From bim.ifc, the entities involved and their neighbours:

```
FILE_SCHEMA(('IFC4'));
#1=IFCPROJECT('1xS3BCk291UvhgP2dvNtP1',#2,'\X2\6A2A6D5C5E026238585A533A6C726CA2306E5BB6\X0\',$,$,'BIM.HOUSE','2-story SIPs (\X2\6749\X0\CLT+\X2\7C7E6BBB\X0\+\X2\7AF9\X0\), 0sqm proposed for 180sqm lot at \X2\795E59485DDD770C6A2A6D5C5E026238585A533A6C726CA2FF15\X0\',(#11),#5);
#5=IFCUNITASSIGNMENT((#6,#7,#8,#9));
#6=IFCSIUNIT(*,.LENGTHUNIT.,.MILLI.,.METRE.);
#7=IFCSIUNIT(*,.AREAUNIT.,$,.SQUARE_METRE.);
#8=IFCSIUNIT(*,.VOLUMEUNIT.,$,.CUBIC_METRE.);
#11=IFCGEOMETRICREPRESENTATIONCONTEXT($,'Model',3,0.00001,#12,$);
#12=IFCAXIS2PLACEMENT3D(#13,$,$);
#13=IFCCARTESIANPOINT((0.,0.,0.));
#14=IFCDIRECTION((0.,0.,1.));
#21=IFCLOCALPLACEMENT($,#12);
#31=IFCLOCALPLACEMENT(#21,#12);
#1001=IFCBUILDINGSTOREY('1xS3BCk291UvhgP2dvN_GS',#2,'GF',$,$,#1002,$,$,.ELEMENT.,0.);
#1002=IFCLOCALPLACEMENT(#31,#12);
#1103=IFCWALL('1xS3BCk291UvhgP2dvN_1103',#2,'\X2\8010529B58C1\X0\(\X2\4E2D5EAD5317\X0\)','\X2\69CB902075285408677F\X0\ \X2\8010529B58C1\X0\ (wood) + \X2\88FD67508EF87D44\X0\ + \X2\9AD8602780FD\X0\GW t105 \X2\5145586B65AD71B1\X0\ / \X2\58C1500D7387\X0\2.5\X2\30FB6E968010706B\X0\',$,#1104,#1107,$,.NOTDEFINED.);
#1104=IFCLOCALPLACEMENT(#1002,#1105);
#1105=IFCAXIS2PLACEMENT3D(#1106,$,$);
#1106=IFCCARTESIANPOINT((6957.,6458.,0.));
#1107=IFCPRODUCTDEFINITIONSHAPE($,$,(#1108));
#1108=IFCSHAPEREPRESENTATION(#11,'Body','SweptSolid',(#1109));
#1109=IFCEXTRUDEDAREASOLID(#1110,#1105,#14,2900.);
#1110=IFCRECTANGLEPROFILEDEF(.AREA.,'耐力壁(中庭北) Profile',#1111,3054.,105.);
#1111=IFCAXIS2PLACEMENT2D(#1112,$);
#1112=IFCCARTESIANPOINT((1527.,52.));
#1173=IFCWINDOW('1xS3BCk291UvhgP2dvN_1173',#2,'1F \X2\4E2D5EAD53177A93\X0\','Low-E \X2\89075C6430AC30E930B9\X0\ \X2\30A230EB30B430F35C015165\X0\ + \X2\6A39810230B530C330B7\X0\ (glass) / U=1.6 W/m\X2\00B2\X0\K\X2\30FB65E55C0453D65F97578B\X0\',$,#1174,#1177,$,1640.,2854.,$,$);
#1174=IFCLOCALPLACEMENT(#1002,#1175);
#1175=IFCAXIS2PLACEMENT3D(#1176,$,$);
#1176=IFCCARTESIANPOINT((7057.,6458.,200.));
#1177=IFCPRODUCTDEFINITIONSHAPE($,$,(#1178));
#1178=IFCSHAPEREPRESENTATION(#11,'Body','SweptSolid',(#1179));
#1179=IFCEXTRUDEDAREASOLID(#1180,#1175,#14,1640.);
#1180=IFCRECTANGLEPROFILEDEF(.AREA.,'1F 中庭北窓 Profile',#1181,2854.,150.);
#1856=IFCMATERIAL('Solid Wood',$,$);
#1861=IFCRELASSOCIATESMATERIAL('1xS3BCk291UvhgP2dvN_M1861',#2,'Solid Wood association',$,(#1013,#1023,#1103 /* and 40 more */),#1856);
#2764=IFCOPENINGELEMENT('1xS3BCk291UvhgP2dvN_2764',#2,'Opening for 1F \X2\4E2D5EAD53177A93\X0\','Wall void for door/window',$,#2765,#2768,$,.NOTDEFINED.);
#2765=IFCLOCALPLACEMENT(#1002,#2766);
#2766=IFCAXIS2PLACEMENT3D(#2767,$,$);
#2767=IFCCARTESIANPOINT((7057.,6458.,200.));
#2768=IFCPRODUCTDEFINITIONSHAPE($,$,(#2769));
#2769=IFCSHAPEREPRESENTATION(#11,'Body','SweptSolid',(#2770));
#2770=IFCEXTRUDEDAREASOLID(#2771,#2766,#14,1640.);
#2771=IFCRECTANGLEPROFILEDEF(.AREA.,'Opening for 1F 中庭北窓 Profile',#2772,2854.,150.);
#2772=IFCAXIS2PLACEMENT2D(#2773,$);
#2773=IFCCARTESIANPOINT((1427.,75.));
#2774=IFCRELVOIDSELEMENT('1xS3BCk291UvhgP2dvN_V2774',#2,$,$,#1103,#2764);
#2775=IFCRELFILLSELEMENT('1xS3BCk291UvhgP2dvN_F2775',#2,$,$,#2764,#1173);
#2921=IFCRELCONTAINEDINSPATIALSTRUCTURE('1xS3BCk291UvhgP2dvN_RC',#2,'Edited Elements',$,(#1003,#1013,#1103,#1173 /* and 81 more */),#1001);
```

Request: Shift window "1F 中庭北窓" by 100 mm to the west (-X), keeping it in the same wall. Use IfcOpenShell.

```python
import ifcopenshell
import ifcopenshell.api.geometry
import ifcopenshell.util.placement

model = ifcopenshell.open("bim.ifc")

window = model.by_guid("1xS3BCk291UvhgP2dvN_1173")
opening = window.FillsVoids[0].RelatingOpeningElement
wall = opening.VoidsElements[0].RelatingBuildingElement

wall_matrix = ifcopenshell.util.placement.get_local_placement(wall.ObjectPlacement)
shift = wall_matrix[:3, 0] * -100.0
before = ifcopenshell.util.placement.get_local_placement(window.ObjectPlacement)[:3, 3].copy()

# The window is not placed relative to its opening, so move both.
for product in (opening, window):
    matrix = ifcopenshell.util.placement.get_local_placement(product.ObjectPlacement)
    matrix[:3, 3] += shift
    ifcopenshell.api.geometry.edit_object_placement(model, product=product, matrix=matrix, is_si=False)

after = ifcopenshell.util.placement.get_local_placement(window.ObjectPlacement)[:3, 3]
print("window moved by", (after - before).round(3) + 0.0)

model.write("bim_updated.ifc")
```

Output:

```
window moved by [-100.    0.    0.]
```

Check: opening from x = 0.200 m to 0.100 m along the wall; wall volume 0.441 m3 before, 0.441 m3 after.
